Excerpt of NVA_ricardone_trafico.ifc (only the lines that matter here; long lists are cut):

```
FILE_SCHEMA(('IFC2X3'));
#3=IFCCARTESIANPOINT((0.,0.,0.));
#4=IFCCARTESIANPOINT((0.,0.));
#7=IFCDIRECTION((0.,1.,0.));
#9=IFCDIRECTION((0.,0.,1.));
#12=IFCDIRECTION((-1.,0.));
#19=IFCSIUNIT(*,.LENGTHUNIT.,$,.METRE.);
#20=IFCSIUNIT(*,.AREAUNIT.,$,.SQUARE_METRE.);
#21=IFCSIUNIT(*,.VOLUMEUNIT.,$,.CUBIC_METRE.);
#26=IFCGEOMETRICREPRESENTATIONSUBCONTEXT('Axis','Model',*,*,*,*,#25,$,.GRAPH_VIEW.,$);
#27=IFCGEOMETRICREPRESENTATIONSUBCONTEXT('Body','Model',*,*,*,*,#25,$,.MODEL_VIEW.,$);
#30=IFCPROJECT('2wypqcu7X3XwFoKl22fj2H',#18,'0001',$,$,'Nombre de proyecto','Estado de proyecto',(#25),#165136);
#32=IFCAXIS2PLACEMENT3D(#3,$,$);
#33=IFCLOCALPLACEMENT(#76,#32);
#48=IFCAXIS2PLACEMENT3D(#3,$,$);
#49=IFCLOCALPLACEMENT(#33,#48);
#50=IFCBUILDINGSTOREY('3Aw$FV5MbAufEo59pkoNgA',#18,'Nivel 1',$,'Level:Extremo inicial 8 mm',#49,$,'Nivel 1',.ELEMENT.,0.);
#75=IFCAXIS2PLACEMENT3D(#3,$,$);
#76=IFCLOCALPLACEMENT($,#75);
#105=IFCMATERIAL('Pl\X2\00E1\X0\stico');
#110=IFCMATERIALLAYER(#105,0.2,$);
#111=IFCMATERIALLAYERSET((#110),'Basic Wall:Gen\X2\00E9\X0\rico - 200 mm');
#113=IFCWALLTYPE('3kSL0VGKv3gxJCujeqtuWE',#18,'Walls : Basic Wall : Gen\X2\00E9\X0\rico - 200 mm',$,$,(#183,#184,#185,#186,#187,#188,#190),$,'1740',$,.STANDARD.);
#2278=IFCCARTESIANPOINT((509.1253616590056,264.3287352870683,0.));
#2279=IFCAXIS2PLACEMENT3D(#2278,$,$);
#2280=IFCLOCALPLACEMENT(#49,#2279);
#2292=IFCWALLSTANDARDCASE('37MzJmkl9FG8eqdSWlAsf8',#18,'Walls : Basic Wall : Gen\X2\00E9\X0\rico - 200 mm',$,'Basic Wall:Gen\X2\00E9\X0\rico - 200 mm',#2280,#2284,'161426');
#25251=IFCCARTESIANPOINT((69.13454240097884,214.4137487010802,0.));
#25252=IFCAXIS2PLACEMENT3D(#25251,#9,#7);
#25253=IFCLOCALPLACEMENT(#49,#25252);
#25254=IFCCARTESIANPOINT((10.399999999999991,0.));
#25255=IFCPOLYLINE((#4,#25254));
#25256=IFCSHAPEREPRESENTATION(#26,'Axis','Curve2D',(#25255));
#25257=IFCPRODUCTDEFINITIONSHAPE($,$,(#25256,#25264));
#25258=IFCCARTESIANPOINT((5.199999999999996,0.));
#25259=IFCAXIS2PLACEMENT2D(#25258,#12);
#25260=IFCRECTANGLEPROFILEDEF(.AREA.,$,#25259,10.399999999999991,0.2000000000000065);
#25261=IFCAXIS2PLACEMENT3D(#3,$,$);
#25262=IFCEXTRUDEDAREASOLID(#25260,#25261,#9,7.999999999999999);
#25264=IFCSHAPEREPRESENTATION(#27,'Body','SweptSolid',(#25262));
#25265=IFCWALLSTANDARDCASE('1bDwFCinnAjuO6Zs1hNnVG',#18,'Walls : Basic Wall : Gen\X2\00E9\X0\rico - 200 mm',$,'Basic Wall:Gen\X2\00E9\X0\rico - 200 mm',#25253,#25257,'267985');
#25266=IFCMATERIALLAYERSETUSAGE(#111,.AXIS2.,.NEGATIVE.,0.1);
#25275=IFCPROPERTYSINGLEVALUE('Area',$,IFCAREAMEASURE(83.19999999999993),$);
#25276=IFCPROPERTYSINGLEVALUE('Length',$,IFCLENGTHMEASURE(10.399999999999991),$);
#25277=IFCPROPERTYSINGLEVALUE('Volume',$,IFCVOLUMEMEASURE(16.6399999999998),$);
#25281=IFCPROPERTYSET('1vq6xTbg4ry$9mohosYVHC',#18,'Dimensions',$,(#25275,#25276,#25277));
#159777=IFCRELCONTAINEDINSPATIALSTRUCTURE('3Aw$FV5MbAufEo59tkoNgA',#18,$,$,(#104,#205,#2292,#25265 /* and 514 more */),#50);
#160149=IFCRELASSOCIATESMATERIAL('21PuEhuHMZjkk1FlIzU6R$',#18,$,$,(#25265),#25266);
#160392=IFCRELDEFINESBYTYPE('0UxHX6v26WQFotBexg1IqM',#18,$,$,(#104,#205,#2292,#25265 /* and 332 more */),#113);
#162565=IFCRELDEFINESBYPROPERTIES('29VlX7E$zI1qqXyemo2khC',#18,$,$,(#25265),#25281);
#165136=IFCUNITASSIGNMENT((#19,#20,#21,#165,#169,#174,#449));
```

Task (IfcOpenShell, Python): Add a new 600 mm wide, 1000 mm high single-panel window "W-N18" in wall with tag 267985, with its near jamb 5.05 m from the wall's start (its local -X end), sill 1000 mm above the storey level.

```python
import numpy as np
import ifcopenshell
import ifcopenshell.api.feature
import ifcopenshell.api.geometry
import ifcopenshell.api.pset
import ifcopenshell.api.root
import ifcopenshell.api.spatial
import ifcopenshell.api.type
import ifcopenshell.geom
import ifcopenshell.util.element
import ifcopenshell.util.placement
import ifcopenshell.util.representation
import ifcopenshell.util.shape
import ifcopenshell.util.unit

model = ifcopenshell.open("NVA_ricardone_trafico.ifc")
unit_scale = ifcopenshell.util.unit.calculate_unit_scale(model)
area_scale = ifcopenshell.util.unit.calculate_unit_scale(model, "AREAUNIT")
volume_scale = ifcopenshell.util.unit.calculate_unit_scale(model, "VOLUMEUNIT")
settings = ifcopenshell.geom.settings()


def volume(element):
    """Net volume in cubic metres, openings subtracted."""
    shape = ifcopenshell.geom.create_shape(settings, element)
    return ifcopenshell.util.shape.get_volume(shape.geometry)


wall = model.by_guid("1bDwFCinnAjuO6Zs1hNnVG")
storey = ifcopenshell.util.element.get_container(wall, ifc_class="IfcBuildingStorey")
context = ifcopenshell.util.representation.get_context(model, "Model", "Body", "MODEL_VIEW")
before = volume(wall)

width, height, from_end, sill = 0.6, 1, 5.05, 1  # metres

# The wall runs along its own X axis, and the end named is its -X end.
wall_shape = ifcopenshell.geom.create_shape(settings, wall)
x, y, z = ifcopenshell.util.shape.get_vertices(wall_shape.geometry).T
start = x.min() + from_end
face, thickness = float(y.min()), float(y.max() - y.min())
wall_matrix = ifcopenshell.util.placement.get_local_placement(wall.ObjectPlacement)
level = ifcopenshell.util.placement.get_local_placement(storey.ObjectPlacement)[2, 3]


def in_wall(x, y):
    """Placement at x, y metres in the wall's axes, at sill height."""
    matrix = wall_matrix.copy()
    matrix[:, 3] = wall_matrix @ np.array([x / unit_scale, y / unit_scale, 0.0, 1.0])
    matrix[2, 3] = level + sill / unit_scale
    return matrix


# Opening: a box that overshoots both wall faces by 50 mm.
opening = ifcopenshell.api.root.create_entity(model, ifc_class="IfcOpeningElement")
box = ifcopenshell.api.geometry.add_wall_representation(
    model, context=context, length=width, height=height, thickness=thickness + 0.1
)
ifcopenshell.api.geometry.assign_representation(model, product=opening, representation=box)
ifcopenshell.api.geometry.edit_object_placement(model, product=opening, matrix=in_wall(start, face - 0.05), is_si=False)
ifcopenshell.api.feature.add_feature(model, feature=opening, element=wall)

window = ifcopenshell.api.root.create_entity(model, ifc_class="IfcWindow", name="W-N18")
window.OverallWidth, window.OverallHeight = width / unit_scale, height / unit_scale
body = ifcopenshell.api.geometry.add_window_representation(
    model,
    context=context,
    overall_width=window.OverallWidth,
    overall_height=window.OverallHeight,
    partition_type="SINGLE_PANEL",
)
ifcopenshell.api.geometry.assign_representation(model, product=window, representation=body)
ifcopenshell.api.spatial.assign_container(model, products=[window], relating_structure=storey)
fills = ifcopenshell.api.feature.add_filling(model, opening=opening, element=window)
fills.OwnerHistory = window.OwnerHistory  # required in IFC2X3

# IFC2X3 keeps the operation on the window style.
style = ifcopenshell.api.root.create_entity(model, ifc_class="IfcWindowStyle", name="W-N18")
style.OperationType, style.ConstructionType = "SINGLE_PANEL", "NOTDEFINED"
style.ParameterTakesPrecedence = style.Sizeable = False
ifcopenshell.api.type.assign_type(model, related_objects=[window], relating_type=style)

# Centre the window in the wall's thickness.
ifcopenshell.api.geometry.edit_object_placement(model, product=window, matrix=in_wall(start, face), is_si=False)
window_shape = ifcopenshell.geom.create_shape(settings, window)
depth = ifcopenshell.util.shape.get_vertices(window_shape.geometry)[:, 1]
offset = face + thickness / 2 - (depth.min() + depth.max()) / 2
ifcopenshell.api.geometry.edit_object_placement(model, product=window, matrix=in_wall(start, offset), is_si=False)

after = volume(wall)

# Update the wall's stored quantities.
pset = model.by_id(ifcopenshell.util.element.get_pset(wall, "Dimensions", should_inherit=False)["id"])
ifcopenshell.api.pset.edit_pset(model, pset=pset, properties={
    "Area": model.create_entity("IfcAreaMeasure", after / thickness / area_scale),
    "Volume": model.create_entity("IfcVolumeMeasure", after / volume_scale),
})

print(f"wall volume {before:.3f} -> {after:.3f} m3")

model.write("NVA_ricardone_trafico-out.ifc")
```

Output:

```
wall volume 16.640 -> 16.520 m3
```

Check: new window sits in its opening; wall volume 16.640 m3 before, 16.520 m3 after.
